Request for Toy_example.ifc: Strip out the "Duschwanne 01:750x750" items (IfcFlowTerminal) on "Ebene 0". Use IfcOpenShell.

First a look at what the model holds.

```python
import ifcopenshell
import ifcopenshell.util.element

model = ifcopenshell.open("Toy_example.ifc")
print(model.schema)
storey = next(s for s in model.by_type("IfcBuildingStorey") if s.Name == "Ebene 0")
terminals = [e for e in ifcopenshell.util.element.get_decomposition(storey) if e.is_a("IfcFlowTerminal")]
seen = {}
for e in terminals:
    element_type = ifcopenshell.util.element.get_type(e)
    name = element_type.Name if element_type not in (None, e) else None
    seen[name] = seen.get(name, 0) + 1
for name, count in sorted(seen.items(), key=str):
    print(count, "x", name)
```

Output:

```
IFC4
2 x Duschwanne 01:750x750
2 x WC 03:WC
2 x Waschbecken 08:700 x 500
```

```python
import ifcopenshell
import ifcopenshell.api.root
import ifcopenshell.util.element

model = ifcopenshell.open("Toy_example.ifc")

storey = next(s for s in model.by_type("IfcBuildingStorey") if s.Name == "Ebene 0")
terminals = [e for e in ifcopenshell.util.element.get_decomposition(storey) if e.is_a("IfcFlowTerminal")]
targets = [e for e in terminals if (t := ifcopenshell.util.element.get_type(e)) not in (None, e) and t.Name == "Duschwanne 01:750x750"]

for e in targets:
    ifcopenshell.api.root.remove_product(model, product=e)
print(len(targets), "removed")

model.write("Toy_example-out.ifc")
```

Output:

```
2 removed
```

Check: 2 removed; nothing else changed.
